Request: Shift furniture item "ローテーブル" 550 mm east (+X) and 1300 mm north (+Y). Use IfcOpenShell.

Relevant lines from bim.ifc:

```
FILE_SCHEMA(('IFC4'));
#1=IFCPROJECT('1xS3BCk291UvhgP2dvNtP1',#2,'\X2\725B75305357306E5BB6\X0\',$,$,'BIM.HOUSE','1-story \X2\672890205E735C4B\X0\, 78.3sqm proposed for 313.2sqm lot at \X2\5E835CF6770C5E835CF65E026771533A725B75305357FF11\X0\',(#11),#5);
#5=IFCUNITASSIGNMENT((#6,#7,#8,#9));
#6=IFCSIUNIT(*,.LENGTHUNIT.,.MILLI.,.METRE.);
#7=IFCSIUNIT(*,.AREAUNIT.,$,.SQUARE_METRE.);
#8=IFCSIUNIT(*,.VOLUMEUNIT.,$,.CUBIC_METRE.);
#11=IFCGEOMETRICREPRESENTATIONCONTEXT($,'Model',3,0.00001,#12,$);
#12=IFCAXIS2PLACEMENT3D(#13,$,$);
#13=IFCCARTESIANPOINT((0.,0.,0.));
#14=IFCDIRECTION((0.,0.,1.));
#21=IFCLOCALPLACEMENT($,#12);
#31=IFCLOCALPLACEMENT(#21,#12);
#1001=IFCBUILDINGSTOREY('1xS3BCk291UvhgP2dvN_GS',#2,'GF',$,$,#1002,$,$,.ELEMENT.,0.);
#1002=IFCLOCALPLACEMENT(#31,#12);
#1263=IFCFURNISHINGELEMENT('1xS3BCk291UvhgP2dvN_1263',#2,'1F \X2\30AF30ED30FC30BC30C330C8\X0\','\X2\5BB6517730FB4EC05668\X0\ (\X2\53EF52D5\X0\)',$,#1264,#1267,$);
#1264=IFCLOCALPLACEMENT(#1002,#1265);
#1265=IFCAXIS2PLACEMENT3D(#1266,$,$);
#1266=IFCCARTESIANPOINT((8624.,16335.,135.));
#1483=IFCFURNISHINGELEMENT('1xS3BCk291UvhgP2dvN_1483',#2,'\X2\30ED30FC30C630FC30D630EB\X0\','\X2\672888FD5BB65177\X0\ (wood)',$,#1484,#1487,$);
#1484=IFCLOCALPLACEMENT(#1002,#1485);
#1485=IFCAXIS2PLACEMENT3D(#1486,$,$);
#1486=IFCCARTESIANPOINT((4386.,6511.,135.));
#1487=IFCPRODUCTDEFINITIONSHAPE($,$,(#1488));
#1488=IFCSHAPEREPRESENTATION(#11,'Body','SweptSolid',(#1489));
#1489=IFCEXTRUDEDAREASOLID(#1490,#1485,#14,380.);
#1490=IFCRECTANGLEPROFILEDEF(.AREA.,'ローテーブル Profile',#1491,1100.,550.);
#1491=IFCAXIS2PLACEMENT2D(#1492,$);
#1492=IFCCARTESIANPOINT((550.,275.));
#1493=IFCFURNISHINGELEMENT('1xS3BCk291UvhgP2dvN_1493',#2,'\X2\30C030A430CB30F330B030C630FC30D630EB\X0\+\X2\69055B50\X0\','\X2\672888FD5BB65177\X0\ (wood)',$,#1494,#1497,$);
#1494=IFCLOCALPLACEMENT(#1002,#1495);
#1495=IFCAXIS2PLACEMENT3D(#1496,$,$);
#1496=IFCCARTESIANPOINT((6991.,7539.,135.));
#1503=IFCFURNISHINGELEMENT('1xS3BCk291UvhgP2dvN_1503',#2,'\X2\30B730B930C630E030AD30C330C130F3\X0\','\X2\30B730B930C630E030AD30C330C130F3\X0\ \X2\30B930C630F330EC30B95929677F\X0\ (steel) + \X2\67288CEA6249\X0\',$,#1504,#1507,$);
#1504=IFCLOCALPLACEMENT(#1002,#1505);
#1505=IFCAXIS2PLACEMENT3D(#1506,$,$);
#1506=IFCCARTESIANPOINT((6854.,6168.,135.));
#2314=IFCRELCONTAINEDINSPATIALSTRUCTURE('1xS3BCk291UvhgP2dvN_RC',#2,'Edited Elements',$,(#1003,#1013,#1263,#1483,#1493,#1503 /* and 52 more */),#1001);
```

```python
import ifcopenshell
import ifcopenshell.api.geometry
import ifcopenshell.util.placement
import ifcopenshell.util.unit

model = ifcopenshell.open("bim.ifc")
unit_scale = ifcopenshell.util.unit.calculate_unit_scale(model)

item = model.by_id(1483)
matrix = ifcopenshell.util.placement.get_local_placement(item.ObjectPlacement)
matrix[0, 3] += 0.55 / unit_scale
matrix[1, 3] += 1.3 / unit_scale
ifcopenshell.api.geometry.edit_object_placement(model, product=item, matrix=matrix, is_si=False)

print(ifcopenshell.util.placement.get_local_placement(item.ObjectPlacement).round(3) + 0.0)

model.write("bim_v2.ifc")
```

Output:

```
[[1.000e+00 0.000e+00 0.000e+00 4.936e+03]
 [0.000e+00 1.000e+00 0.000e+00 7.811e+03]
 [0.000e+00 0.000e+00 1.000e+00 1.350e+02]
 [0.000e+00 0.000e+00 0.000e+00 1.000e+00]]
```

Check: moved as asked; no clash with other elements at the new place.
